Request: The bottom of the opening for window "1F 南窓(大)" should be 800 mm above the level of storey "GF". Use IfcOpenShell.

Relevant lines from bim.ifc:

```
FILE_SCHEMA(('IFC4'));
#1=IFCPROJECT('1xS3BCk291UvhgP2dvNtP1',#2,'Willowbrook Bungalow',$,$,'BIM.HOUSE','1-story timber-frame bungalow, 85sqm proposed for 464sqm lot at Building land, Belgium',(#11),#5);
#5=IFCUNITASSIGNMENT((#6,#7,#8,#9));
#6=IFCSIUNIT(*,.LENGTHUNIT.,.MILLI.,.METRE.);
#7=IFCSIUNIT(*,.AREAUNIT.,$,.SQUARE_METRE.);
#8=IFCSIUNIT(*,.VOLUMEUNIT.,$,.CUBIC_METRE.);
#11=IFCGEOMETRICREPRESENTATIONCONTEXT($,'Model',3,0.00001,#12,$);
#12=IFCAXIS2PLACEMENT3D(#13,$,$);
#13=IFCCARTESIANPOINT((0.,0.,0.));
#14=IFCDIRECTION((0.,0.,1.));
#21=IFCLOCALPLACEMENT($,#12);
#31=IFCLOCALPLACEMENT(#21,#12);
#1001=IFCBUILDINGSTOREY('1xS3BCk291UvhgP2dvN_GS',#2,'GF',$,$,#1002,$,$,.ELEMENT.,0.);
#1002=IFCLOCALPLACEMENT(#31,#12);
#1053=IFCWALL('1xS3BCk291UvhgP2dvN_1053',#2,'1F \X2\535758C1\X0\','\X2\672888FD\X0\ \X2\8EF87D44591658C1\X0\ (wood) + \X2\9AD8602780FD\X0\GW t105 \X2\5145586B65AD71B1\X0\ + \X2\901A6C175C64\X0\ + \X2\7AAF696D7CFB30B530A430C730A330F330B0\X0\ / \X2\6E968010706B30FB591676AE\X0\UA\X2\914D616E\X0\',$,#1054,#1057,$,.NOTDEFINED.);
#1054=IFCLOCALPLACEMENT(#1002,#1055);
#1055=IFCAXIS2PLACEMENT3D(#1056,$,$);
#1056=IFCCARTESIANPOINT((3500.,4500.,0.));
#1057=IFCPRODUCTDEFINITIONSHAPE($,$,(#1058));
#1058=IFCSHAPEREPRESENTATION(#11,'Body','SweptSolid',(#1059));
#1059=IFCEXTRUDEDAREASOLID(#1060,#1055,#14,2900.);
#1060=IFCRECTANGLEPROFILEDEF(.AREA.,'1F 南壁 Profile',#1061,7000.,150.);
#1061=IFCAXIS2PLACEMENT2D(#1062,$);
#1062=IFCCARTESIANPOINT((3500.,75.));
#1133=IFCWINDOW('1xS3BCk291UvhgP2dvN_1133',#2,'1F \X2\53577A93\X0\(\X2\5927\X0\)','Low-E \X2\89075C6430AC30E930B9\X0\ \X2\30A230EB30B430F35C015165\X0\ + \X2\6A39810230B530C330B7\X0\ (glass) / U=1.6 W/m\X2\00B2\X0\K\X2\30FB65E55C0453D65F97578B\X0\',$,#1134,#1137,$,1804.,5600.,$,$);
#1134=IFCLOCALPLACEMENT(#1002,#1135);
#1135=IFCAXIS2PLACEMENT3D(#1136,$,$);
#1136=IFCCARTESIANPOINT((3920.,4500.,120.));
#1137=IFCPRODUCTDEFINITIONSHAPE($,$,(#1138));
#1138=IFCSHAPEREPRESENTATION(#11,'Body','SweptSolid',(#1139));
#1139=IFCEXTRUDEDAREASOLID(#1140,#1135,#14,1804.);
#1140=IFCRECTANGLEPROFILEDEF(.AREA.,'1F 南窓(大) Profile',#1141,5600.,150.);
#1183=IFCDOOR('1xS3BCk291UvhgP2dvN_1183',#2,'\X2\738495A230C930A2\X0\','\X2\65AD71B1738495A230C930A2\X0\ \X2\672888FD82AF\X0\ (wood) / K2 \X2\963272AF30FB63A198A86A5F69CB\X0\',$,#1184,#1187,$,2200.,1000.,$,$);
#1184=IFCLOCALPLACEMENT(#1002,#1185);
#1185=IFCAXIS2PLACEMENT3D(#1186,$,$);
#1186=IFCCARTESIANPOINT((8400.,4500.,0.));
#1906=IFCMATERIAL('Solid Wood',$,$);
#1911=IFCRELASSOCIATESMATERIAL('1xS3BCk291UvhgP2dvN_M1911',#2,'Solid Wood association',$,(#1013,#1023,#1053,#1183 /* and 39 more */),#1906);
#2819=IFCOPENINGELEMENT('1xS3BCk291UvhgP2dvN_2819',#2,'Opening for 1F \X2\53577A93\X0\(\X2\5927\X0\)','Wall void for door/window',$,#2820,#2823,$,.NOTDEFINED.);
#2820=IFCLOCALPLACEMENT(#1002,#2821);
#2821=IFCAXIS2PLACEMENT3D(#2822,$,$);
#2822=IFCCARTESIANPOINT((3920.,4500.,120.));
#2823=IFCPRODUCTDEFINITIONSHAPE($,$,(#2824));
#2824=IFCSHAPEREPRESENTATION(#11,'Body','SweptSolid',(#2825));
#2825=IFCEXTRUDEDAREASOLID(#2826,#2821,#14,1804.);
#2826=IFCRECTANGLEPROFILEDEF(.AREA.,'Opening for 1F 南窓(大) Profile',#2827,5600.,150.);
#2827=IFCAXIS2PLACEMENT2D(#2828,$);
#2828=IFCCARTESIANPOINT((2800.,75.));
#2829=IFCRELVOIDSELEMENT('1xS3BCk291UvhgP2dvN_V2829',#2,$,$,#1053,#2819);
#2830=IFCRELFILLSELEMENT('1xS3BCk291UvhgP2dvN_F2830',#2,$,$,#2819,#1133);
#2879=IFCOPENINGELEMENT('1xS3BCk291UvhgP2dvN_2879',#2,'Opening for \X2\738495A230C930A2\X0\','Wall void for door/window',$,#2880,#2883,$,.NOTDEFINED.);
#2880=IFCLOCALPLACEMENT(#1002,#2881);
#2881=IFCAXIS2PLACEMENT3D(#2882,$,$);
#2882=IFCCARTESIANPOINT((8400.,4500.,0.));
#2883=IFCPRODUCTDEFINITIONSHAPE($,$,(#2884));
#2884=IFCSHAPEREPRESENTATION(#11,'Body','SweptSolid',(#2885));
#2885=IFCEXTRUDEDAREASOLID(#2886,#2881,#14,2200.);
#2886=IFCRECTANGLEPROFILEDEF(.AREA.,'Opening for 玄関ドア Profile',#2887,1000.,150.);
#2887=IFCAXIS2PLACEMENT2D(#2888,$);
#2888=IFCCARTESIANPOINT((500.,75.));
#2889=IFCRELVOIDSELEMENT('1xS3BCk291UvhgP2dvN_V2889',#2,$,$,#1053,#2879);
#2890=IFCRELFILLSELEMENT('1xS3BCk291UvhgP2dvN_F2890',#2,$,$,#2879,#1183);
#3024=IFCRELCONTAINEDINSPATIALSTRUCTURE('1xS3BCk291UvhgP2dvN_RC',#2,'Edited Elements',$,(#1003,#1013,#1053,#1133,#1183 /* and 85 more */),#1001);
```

```python
import numpy as np
import ifcopenshell
import ifcopenshell.api.geometry
import ifcopenshell.geom
import ifcopenshell.util.element
import ifcopenshell.util.placement
import ifcopenshell.util.shape
import ifcopenshell.util.unit

model = ifcopenshell.open("bim.ifc")
unit_scale = ifcopenshell.util.unit.calculate_unit_scale(model)

window = model.by_guid("1xS3BCk291UvhgP2dvN_1133")
opening = window.FillsVoids[0].RelatingOpeningElement
storey = ifcopenshell.util.element.get_container(window, ifc_class="IfcBuildingStorey")
level = ifcopenshell.util.placement.get_local_placement(storey.ObjectPlacement)[2, 3]

# The opening's origin need not be at the sill, so measure its lowest point.
shape = ifcopenshell.geom.create_shape(ifcopenshell.geom.settings(), opening)
bottom = ifcopenshell.util.shape.get_shape_bottom_elevation(shape, shape.geometry) / unit_scale
dz = level + 800.0 - bottom

shift = np.array([0.0, 0.0, dz])
# The window is not placed relative to its opening, so move both.
for product in (opening, window):
    matrix = ifcopenshell.util.placement.get_local_placement(product.ObjectPlacement)
    matrix[:3, 3] += shift
    ifcopenshell.api.geometry.edit_object_placement(model, product=product, matrix=matrix, is_si=False)

print(f"moved by {dz * unit_scale:+.3f} m")

model.write("bim_rev.ifc")
```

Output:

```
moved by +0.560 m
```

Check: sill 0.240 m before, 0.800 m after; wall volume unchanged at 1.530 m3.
